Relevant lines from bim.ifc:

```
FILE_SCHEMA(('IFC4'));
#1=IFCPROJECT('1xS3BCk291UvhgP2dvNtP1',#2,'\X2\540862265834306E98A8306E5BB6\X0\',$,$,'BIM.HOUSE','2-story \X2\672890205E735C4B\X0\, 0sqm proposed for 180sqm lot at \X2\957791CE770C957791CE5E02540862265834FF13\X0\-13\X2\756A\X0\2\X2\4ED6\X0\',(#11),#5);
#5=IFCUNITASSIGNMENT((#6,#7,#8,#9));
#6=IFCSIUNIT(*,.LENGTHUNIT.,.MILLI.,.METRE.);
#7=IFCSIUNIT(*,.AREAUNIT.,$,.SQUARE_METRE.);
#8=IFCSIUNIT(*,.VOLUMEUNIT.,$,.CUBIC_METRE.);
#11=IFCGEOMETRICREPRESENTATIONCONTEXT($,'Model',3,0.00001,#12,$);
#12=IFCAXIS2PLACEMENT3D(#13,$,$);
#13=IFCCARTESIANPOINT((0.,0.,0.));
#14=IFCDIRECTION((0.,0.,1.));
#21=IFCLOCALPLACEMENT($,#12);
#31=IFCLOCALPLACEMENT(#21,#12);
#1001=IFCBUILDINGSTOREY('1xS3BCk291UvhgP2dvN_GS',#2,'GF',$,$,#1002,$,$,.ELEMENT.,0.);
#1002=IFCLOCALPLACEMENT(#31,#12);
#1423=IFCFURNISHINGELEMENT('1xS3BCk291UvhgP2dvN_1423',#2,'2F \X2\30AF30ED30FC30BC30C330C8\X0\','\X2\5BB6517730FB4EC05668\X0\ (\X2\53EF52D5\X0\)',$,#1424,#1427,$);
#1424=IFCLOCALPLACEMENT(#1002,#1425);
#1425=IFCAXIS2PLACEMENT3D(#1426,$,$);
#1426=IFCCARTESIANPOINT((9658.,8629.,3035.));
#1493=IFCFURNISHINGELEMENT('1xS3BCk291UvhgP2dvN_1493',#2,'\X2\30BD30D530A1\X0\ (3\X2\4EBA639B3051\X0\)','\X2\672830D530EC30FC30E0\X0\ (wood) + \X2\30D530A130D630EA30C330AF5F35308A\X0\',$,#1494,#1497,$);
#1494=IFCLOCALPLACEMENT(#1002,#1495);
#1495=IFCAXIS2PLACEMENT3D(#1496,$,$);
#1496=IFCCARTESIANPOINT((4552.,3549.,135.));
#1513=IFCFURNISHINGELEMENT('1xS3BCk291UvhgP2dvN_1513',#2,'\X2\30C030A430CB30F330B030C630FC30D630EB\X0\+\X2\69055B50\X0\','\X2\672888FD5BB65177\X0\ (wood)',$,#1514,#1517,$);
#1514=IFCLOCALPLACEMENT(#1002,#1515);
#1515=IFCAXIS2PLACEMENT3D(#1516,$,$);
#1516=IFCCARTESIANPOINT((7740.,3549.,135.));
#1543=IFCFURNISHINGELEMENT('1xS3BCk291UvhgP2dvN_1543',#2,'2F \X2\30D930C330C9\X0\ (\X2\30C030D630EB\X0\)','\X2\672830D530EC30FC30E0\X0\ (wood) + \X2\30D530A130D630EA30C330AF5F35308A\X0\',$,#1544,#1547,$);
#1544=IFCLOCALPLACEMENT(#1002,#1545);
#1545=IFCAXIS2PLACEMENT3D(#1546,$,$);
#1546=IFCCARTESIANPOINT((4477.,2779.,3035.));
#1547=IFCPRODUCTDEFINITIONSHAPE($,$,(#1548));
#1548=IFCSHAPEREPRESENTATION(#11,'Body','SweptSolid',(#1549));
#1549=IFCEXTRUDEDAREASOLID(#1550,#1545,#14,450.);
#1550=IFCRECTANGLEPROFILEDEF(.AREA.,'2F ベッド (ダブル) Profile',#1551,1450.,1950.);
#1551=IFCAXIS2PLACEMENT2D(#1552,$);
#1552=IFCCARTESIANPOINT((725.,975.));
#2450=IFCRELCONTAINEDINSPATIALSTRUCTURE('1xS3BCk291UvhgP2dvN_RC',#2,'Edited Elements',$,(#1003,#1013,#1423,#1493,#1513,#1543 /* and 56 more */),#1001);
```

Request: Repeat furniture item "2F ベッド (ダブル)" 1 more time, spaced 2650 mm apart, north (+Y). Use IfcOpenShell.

```python
import numpy as np
import ifcopenshell
import ifcopenshell.api.geometry
import ifcopenshell.api.root
import ifcopenshell.util.element
import ifcopenshell.util.placement

model = ifcopenshell.open("bim.ifc")


def reuse_history(source, copy):
    """copy_class also copies each property set's owner history, people and application; keep the originals."""
    for rel in copy.IsDefinedBy:
        if rel.is_a("IfcRelDefinesByProperties") and (history := rel.RelatingPropertyDefinition.OwnerHistory):
            rel.RelatingPropertyDefinition.OwnerHistory = source.OwnerHistory
            ifcopenshell.util.element.remove_deep2(model, history)


source = model.by_guid("1xS3BCk291UvhgP2dvN_1543")
base = ifcopenshell.util.placement.get_local_placement(source.ObjectPlacement)
step = np.array([0.0, 1.0, 0.0]) * 2650.0

for i in range(1, 2):
    copy = ifcopenshell.api.root.copy_class(model, product=source)
    copy.Representation = ifcopenshell.util.element.copy_deep(
        model, source.Representation, exclude=["IfcGeometricRepresentationContext", "IfcRepresentationMap"]
    )
    reuse_history(source, copy)
    matrix = base.copy()
    matrix[:3, 3] += i * step
    print("added at", matrix[:3, 3].round(3) + 0.0)
    ifcopenshell.api.geometry.edit_object_placement(model, product=copy, matrix=matrix, is_si=False)

model.write("bim_updated.ifc")
```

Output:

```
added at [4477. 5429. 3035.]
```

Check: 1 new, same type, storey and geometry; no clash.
